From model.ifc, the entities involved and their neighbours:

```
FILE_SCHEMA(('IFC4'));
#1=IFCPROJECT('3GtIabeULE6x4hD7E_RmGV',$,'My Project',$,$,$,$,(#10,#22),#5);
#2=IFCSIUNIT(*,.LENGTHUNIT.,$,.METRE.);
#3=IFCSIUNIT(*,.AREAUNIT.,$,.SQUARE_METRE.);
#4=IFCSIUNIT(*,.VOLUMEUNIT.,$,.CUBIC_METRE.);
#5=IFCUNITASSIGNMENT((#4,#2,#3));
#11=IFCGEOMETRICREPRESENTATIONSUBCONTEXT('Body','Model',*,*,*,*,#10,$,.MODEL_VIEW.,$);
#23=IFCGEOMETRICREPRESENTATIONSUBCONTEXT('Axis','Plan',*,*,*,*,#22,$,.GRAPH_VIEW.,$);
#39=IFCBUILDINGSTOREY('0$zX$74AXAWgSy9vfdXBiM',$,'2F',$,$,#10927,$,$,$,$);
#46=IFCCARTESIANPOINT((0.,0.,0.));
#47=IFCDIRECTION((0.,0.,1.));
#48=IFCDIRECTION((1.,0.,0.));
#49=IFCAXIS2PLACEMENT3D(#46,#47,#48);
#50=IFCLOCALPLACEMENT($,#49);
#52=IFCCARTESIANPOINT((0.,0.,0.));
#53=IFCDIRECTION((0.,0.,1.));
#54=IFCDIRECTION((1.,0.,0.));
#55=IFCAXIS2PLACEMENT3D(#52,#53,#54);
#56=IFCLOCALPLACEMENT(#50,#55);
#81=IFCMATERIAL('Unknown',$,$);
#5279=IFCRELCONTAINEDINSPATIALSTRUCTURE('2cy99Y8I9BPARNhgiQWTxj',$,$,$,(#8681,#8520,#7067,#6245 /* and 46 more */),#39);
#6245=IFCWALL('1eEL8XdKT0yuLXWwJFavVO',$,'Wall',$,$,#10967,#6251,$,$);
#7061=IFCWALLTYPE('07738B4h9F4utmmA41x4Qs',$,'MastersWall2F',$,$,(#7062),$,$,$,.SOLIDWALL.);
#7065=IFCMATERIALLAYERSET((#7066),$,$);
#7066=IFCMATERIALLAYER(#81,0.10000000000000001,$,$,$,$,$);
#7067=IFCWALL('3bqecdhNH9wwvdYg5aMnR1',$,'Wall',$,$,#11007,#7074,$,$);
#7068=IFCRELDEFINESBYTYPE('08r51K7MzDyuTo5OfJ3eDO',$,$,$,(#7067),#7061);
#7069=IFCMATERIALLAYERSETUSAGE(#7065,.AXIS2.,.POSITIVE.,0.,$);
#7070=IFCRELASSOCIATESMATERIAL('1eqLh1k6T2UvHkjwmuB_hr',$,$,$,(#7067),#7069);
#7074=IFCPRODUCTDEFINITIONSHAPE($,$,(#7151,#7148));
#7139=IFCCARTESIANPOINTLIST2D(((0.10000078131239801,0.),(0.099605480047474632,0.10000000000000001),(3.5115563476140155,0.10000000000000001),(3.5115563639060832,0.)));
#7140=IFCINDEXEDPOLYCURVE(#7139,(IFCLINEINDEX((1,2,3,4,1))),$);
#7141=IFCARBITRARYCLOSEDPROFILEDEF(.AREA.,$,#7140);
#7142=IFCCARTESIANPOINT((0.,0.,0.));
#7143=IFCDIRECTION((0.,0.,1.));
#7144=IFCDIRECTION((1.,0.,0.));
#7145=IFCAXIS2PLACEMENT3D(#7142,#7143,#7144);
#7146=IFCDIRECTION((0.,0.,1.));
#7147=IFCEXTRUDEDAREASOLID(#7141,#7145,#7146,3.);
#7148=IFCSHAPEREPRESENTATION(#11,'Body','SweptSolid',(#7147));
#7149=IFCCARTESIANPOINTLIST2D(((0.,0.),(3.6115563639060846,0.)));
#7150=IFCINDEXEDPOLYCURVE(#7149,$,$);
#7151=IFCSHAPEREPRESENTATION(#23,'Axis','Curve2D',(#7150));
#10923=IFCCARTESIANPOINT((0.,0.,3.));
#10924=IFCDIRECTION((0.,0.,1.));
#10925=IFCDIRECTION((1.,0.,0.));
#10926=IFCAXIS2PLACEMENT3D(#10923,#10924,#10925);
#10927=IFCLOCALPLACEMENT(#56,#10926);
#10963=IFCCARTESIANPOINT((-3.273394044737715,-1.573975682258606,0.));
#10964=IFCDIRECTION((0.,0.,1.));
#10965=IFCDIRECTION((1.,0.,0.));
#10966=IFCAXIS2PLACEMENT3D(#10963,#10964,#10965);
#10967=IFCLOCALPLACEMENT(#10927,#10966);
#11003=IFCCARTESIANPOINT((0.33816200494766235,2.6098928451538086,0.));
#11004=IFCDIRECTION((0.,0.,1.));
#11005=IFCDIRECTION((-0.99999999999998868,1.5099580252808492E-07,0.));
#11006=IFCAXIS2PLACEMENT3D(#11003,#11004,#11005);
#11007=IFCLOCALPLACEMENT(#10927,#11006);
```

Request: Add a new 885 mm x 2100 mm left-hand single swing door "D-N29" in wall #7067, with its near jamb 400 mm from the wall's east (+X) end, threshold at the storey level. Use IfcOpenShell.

```python
import numpy as np
import ifcopenshell
import ifcopenshell.api.feature
import ifcopenshell.api.geometry
import ifcopenshell.api.root
import ifcopenshell.api.spatial
import ifcopenshell.geom
import ifcopenshell.util.element
import ifcopenshell.util.placement
import ifcopenshell.util.representation
import ifcopenshell.util.shape
import ifcopenshell.util.unit

model = ifcopenshell.open("model.ifc")
unit_scale = ifcopenshell.util.unit.calculate_unit_scale(model)
settings = ifcopenshell.geom.settings()


def volume(element):
    """Net volume in cubic metres, openings subtracted."""
    shape = ifcopenshell.geom.create_shape(settings, element)
    return ifcopenshell.util.shape.get_volume(shape.geometry)


wall = model.by_guid("3bqecdhNH9wwvdYg5aMnR1")
storey = ifcopenshell.util.element.get_container(wall, ifc_class="IfcBuildingStorey")
context = ifcopenshell.util.representation.get_context(model, "Model", "Body", "MODEL_VIEW")
before = volume(wall)

width, height, from_end, sill = 0.885, 2.1, 0.4, 0.0  # metres

# The wall runs along its own X axis, and the end named is its -X end.
wall_shape = ifcopenshell.geom.create_shape(settings, wall)
x, y, z = ifcopenshell.util.shape.get_vertices(wall_shape.geometry).T
start = x.min() + from_end
face, thickness = float(y.min()), float(y.max() - y.min())
wall_matrix = ifcopenshell.util.placement.get_local_placement(wall.ObjectPlacement)
level = ifcopenshell.util.placement.get_local_placement(storey.ObjectPlacement)[2, 3]


def in_wall(x, y):
    """Placement at x, y metres in the wall's axes, at sill height."""
    matrix = wall_matrix.copy()
    matrix[:, 3] = wall_matrix @ np.array([x / unit_scale, y / unit_scale, 0.0, 1.0])
    matrix[2, 3] = level + sill / unit_scale
    return matrix


# Opening: a box that overshoots both wall faces by 50 mm.
opening = ifcopenshell.api.root.create_entity(model, ifc_class="IfcOpeningElement", predefined_type="OPENING")
box = ifcopenshell.api.geometry.add_wall_representation(
    model, context=context, length=width, height=height, thickness=thickness + 0.1
)
ifcopenshell.api.geometry.assign_representation(model, product=opening, representation=box)
ifcopenshell.api.geometry.edit_object_placement(model, product=opening, matrix=in_wall(start, face - 0.05), is_si=False)
ifcopenshell.api.feature.add_feature(model, feature=opening, element=wall)

door = ifcopenshell.api.root.create_entity(model, ifc_class="IfcDoor", name="D-N29", predefined_type="DOOR")
door.OverallWidth, door.OverallHeight = width / unit_scale, height / unit_scale
door.OperationType = "SINGLE_SWING_LEFT"
body = ifcopenshell.api.geometry.add_door_representation(
    model,
    context=context,
    overall_width=door.OverallWidth,
    overall_height=door.OverallHeight,
    operation_type="SINGLE_SWING_LEFT",
    lining_properties={"LiningDepth": thickness / unit_scale, "ThresholdDepth": thickness / unit_scale},
)
ifcopenshell.api.geometry.assign_representation(model, product=door, representation=body)
ifcopenshell.api.spatial.assign_container(model, products=[door], relating_structure=storey)
ifcopenshell.api.feature.add_filling(model, opening=opening, element=door)

# The lining spans the wall, so the door starts at the wall face.
ifcopenshell.api.geometry.edit_object_placement(model, product=door, matrix=in_wall(start, face), is_si=False)

after = volume(wall)

print(f"wall volume {before:.3f} -> {after:.3f} m3")

model.write("model_edited.ifc")
```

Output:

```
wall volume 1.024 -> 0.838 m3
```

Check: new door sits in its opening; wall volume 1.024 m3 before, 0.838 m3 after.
